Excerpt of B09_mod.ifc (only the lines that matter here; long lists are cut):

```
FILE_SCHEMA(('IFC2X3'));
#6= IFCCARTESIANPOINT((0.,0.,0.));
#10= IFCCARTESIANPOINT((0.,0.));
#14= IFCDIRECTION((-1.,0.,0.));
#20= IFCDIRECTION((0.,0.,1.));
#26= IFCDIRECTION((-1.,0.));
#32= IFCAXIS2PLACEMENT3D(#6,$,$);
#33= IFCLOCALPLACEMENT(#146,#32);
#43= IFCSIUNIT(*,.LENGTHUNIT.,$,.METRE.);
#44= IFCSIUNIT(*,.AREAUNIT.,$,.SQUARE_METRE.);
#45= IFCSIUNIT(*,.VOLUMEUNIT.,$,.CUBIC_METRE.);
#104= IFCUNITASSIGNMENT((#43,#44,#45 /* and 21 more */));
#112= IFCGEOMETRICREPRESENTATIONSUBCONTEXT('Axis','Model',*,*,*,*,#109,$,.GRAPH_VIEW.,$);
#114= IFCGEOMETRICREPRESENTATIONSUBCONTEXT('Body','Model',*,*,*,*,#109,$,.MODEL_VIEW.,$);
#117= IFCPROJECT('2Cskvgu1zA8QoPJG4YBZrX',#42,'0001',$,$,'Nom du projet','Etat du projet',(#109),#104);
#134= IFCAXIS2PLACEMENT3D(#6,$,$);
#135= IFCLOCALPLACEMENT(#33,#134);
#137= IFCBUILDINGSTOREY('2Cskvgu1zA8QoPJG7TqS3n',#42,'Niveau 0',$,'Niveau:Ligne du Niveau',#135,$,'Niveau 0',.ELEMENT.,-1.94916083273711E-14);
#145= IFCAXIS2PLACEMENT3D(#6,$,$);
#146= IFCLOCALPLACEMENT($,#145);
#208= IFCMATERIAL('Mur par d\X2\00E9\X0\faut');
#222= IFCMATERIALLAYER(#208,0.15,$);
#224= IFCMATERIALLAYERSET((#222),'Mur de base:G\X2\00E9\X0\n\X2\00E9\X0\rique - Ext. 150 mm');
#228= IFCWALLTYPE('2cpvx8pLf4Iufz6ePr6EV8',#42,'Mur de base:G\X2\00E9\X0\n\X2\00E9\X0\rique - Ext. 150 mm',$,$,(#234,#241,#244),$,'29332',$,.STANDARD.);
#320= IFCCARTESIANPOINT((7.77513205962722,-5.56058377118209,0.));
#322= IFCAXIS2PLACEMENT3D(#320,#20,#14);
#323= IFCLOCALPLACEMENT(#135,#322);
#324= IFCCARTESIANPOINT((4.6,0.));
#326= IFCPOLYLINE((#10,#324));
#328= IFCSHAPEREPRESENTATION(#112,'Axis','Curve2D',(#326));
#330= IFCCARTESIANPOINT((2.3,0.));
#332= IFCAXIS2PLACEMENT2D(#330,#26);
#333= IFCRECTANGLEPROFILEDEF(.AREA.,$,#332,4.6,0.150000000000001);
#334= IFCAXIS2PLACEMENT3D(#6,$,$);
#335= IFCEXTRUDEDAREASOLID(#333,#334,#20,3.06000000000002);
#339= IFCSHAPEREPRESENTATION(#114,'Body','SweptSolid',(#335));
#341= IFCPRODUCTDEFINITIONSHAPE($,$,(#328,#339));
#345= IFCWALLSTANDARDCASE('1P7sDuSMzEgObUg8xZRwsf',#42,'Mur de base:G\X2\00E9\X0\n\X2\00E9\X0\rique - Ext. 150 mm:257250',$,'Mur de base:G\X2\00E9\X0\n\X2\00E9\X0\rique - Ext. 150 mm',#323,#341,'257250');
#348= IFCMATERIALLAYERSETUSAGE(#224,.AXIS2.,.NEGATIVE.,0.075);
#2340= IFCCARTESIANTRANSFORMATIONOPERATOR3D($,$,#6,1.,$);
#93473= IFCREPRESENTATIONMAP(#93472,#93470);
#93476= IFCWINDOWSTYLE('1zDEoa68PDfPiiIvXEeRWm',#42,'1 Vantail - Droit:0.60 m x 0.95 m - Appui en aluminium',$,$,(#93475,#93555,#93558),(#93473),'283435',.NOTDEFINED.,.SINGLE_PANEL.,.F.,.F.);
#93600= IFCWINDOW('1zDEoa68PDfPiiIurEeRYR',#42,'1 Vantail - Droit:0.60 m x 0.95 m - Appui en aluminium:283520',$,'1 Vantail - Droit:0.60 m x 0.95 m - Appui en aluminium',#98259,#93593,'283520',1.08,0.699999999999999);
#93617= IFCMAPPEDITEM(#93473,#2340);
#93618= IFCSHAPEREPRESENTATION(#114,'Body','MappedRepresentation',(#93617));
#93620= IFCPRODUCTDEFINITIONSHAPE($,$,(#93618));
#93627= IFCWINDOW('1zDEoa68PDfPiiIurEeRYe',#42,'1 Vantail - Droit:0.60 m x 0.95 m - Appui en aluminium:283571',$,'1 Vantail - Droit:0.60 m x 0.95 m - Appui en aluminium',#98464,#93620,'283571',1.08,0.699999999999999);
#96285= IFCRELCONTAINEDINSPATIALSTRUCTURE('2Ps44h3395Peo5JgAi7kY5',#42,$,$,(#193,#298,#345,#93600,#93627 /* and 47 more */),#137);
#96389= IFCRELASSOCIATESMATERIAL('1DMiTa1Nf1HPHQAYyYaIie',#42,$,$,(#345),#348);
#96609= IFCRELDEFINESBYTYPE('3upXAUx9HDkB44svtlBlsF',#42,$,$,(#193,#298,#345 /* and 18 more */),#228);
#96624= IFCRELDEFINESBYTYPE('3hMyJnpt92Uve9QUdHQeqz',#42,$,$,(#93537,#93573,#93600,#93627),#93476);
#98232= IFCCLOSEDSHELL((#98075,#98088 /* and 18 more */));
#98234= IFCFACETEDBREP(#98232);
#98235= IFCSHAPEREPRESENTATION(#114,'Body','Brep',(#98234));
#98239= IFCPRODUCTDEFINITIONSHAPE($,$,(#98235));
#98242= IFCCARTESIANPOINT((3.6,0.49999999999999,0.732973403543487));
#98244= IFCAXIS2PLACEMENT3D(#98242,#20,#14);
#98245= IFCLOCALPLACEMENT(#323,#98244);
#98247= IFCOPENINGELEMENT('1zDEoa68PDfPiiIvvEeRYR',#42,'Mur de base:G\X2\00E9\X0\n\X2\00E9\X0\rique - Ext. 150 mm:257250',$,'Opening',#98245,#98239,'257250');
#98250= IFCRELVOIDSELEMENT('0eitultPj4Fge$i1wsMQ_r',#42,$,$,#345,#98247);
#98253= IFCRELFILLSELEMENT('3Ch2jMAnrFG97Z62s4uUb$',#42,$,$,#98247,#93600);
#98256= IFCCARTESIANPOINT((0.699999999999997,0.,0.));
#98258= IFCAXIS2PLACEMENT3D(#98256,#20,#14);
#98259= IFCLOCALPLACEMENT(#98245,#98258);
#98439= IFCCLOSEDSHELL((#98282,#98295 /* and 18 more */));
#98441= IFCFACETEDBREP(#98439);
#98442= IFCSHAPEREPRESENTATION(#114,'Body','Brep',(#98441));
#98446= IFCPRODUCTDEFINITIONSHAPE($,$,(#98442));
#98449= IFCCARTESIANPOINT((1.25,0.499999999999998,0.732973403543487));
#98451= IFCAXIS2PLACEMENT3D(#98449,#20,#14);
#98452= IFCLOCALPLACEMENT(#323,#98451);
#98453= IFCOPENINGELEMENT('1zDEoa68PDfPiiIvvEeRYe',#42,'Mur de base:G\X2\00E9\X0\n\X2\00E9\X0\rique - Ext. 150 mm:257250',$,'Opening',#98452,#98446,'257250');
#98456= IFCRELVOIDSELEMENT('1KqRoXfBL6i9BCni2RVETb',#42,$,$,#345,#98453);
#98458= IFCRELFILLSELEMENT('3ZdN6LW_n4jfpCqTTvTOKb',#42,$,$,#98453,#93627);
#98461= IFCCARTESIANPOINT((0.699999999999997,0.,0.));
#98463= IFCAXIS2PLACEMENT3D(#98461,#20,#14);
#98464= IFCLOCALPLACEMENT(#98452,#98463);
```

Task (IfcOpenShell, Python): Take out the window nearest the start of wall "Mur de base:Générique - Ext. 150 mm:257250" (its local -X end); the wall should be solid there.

```python
import ifcopenshell
import ifcopenshell.api.feature
import ifcopenshell.api.root
import ifcopenshell.geom
import ifcopenshell.util.shape

model = ifcopenshell.open("B09_mod.ifc")
settings = ifcopenshell.geom.settings()


def volume(element):
    """Net volume in cubic metres, openings subtracted."""
    shape = ifcopenshell.geom.create_shape(settings, element)
    return ifcopenshell.util.shape.get_volume(shape.geometry)


window = model.by_guid("1zDEoa68PDfPiiIurEeRYe")
opening = window.FillsVoids[0].RelatingOpeningElement
wall = opening.VoidsElements[0].RelatingBuildingElement
before = volume(wall)

ifcopenshell.api.root.remove_product(model, product=window)
ifcopenshell.api.feature.remove_feature(model, feature=opening)

after = volume(wall)

print(f"wall volume {before:.3f} -> {after:.3f} m3")

model.write("B09_mod_updated.ifc")
```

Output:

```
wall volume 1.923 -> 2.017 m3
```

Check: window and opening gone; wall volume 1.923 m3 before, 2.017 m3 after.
